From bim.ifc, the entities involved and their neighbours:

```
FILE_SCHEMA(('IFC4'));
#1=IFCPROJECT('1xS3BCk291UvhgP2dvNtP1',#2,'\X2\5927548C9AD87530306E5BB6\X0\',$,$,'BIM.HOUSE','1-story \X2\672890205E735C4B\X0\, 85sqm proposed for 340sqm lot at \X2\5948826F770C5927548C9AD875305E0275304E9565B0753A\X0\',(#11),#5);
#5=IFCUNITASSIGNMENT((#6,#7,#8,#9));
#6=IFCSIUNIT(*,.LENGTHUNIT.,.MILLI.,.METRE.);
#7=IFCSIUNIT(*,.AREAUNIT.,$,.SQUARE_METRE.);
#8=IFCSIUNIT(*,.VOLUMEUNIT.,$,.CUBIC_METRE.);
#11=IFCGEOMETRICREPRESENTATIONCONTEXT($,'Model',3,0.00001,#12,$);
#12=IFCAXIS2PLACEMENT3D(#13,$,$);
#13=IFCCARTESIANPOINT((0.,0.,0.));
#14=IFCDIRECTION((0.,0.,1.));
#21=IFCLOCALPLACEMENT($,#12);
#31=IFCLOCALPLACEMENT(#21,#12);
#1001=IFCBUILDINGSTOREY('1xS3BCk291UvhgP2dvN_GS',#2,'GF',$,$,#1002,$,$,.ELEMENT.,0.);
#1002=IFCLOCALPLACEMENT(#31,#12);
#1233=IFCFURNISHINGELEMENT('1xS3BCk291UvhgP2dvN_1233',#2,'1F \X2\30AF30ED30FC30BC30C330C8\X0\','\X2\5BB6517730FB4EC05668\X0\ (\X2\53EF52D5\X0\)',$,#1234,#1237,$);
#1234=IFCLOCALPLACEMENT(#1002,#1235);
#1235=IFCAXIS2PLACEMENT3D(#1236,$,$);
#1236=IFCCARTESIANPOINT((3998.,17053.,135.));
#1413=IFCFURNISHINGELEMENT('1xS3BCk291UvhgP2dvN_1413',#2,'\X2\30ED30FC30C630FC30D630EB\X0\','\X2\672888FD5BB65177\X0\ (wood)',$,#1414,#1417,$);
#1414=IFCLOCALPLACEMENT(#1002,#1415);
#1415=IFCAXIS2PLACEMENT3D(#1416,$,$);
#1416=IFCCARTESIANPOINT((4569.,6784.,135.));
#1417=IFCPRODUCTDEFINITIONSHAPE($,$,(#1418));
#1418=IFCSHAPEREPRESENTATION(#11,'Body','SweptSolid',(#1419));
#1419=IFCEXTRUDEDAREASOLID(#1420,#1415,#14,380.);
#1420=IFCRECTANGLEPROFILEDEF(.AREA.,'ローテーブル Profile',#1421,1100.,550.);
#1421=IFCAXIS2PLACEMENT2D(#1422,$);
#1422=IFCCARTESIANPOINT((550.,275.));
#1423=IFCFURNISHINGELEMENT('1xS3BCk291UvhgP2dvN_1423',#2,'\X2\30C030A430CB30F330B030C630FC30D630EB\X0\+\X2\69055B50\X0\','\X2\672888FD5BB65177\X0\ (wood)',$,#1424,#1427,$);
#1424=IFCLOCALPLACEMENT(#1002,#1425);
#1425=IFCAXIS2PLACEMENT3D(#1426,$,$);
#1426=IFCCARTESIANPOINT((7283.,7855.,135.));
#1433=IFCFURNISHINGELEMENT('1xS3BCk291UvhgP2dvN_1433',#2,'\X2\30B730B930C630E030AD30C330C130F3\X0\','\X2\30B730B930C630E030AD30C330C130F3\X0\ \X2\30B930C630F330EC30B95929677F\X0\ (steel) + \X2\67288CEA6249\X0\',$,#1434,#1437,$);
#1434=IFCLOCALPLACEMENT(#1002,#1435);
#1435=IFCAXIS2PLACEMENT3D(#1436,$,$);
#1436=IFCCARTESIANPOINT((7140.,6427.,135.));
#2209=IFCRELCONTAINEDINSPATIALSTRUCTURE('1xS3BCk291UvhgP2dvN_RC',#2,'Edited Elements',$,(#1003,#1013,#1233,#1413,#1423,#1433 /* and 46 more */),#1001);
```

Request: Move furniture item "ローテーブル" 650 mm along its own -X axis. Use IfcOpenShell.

```python
import ifcopenshell
import ifcopenshell.api.geometry
import ifcopenshell.util.placement
import ifcopenshell.util.unit

model = ifcopenshell.open("bim.ifc")
unit_scale = ifcopenshell.util.unit.calculate_unit_scale(model)

item = model.by_id(1413)
matrix = ifcopenshell.util.placement.get_local_placement(item.ObjectPlacement)
matrix[:3, 3] -= matrix[:3, 0] * 0.65 / unit_scale
ifcopenshell.api.geometry.edit_object_placement(model, product=item, matrix=matrix, is_si=False)

print(ifcopenshell.util.placement.get_local_placement(item.ObjectPlacement).round(3) + 0.0)

model.write("bim_rev.ifc")
```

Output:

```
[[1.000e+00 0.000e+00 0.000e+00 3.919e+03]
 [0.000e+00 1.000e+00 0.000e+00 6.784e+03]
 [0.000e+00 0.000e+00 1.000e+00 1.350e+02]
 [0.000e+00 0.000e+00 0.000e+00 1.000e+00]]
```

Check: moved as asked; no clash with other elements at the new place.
